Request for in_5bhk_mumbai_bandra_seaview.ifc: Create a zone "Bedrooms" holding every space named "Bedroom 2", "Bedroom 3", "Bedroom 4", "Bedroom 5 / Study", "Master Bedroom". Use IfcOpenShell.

First a look at what the model holds.

```python
import ifcopenshell

model = ifcopenshell.open("in_5bhk_mumbai_bandra_seaview.ifc")
print(model.schema)
seen = {}
for space in model.by_type("IfcSpace"):
    seen[space.LongName] = seen.get(space.LongName, 0) + 1
for name, count in sorted(seen.items(), key=str):
    print(count, "x", name)
print("zones:", [z.Name for z in model.by_type("IfcZone")][:20])
```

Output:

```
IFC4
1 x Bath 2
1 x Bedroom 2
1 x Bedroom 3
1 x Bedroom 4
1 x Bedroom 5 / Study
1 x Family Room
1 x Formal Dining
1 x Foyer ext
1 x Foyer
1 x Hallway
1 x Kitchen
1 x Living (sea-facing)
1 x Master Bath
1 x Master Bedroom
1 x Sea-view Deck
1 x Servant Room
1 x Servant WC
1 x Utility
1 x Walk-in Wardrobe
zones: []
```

```python
import ifcopenshell
import ifcopenshell.api.group
import ifcopenshell.api.root

model = ifcopenshell.open("in_5bhk_mumbai_bandra_seaview.ifc")

names = {"Bedroom 2", "Bedroom 3", "Bedroom 4", "Bedroom 5 / Study", "Master Bedroom"}
spaces = [s for s in model.by_type("IfcSpace") if s.LongName in names]

zone = ifcopenshell.api.root.create_entity(model, ifc_class="IfcZone", name="Bedrooms")
ifcopenshell.api.group.assign_group(model, products=spaces, group=zone)
print(len(spaces), "spaces in", zone.Name)

model.write("in_5bhk_mumbai_bandra_seaview-out.ifc")
```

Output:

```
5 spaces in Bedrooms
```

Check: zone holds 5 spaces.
